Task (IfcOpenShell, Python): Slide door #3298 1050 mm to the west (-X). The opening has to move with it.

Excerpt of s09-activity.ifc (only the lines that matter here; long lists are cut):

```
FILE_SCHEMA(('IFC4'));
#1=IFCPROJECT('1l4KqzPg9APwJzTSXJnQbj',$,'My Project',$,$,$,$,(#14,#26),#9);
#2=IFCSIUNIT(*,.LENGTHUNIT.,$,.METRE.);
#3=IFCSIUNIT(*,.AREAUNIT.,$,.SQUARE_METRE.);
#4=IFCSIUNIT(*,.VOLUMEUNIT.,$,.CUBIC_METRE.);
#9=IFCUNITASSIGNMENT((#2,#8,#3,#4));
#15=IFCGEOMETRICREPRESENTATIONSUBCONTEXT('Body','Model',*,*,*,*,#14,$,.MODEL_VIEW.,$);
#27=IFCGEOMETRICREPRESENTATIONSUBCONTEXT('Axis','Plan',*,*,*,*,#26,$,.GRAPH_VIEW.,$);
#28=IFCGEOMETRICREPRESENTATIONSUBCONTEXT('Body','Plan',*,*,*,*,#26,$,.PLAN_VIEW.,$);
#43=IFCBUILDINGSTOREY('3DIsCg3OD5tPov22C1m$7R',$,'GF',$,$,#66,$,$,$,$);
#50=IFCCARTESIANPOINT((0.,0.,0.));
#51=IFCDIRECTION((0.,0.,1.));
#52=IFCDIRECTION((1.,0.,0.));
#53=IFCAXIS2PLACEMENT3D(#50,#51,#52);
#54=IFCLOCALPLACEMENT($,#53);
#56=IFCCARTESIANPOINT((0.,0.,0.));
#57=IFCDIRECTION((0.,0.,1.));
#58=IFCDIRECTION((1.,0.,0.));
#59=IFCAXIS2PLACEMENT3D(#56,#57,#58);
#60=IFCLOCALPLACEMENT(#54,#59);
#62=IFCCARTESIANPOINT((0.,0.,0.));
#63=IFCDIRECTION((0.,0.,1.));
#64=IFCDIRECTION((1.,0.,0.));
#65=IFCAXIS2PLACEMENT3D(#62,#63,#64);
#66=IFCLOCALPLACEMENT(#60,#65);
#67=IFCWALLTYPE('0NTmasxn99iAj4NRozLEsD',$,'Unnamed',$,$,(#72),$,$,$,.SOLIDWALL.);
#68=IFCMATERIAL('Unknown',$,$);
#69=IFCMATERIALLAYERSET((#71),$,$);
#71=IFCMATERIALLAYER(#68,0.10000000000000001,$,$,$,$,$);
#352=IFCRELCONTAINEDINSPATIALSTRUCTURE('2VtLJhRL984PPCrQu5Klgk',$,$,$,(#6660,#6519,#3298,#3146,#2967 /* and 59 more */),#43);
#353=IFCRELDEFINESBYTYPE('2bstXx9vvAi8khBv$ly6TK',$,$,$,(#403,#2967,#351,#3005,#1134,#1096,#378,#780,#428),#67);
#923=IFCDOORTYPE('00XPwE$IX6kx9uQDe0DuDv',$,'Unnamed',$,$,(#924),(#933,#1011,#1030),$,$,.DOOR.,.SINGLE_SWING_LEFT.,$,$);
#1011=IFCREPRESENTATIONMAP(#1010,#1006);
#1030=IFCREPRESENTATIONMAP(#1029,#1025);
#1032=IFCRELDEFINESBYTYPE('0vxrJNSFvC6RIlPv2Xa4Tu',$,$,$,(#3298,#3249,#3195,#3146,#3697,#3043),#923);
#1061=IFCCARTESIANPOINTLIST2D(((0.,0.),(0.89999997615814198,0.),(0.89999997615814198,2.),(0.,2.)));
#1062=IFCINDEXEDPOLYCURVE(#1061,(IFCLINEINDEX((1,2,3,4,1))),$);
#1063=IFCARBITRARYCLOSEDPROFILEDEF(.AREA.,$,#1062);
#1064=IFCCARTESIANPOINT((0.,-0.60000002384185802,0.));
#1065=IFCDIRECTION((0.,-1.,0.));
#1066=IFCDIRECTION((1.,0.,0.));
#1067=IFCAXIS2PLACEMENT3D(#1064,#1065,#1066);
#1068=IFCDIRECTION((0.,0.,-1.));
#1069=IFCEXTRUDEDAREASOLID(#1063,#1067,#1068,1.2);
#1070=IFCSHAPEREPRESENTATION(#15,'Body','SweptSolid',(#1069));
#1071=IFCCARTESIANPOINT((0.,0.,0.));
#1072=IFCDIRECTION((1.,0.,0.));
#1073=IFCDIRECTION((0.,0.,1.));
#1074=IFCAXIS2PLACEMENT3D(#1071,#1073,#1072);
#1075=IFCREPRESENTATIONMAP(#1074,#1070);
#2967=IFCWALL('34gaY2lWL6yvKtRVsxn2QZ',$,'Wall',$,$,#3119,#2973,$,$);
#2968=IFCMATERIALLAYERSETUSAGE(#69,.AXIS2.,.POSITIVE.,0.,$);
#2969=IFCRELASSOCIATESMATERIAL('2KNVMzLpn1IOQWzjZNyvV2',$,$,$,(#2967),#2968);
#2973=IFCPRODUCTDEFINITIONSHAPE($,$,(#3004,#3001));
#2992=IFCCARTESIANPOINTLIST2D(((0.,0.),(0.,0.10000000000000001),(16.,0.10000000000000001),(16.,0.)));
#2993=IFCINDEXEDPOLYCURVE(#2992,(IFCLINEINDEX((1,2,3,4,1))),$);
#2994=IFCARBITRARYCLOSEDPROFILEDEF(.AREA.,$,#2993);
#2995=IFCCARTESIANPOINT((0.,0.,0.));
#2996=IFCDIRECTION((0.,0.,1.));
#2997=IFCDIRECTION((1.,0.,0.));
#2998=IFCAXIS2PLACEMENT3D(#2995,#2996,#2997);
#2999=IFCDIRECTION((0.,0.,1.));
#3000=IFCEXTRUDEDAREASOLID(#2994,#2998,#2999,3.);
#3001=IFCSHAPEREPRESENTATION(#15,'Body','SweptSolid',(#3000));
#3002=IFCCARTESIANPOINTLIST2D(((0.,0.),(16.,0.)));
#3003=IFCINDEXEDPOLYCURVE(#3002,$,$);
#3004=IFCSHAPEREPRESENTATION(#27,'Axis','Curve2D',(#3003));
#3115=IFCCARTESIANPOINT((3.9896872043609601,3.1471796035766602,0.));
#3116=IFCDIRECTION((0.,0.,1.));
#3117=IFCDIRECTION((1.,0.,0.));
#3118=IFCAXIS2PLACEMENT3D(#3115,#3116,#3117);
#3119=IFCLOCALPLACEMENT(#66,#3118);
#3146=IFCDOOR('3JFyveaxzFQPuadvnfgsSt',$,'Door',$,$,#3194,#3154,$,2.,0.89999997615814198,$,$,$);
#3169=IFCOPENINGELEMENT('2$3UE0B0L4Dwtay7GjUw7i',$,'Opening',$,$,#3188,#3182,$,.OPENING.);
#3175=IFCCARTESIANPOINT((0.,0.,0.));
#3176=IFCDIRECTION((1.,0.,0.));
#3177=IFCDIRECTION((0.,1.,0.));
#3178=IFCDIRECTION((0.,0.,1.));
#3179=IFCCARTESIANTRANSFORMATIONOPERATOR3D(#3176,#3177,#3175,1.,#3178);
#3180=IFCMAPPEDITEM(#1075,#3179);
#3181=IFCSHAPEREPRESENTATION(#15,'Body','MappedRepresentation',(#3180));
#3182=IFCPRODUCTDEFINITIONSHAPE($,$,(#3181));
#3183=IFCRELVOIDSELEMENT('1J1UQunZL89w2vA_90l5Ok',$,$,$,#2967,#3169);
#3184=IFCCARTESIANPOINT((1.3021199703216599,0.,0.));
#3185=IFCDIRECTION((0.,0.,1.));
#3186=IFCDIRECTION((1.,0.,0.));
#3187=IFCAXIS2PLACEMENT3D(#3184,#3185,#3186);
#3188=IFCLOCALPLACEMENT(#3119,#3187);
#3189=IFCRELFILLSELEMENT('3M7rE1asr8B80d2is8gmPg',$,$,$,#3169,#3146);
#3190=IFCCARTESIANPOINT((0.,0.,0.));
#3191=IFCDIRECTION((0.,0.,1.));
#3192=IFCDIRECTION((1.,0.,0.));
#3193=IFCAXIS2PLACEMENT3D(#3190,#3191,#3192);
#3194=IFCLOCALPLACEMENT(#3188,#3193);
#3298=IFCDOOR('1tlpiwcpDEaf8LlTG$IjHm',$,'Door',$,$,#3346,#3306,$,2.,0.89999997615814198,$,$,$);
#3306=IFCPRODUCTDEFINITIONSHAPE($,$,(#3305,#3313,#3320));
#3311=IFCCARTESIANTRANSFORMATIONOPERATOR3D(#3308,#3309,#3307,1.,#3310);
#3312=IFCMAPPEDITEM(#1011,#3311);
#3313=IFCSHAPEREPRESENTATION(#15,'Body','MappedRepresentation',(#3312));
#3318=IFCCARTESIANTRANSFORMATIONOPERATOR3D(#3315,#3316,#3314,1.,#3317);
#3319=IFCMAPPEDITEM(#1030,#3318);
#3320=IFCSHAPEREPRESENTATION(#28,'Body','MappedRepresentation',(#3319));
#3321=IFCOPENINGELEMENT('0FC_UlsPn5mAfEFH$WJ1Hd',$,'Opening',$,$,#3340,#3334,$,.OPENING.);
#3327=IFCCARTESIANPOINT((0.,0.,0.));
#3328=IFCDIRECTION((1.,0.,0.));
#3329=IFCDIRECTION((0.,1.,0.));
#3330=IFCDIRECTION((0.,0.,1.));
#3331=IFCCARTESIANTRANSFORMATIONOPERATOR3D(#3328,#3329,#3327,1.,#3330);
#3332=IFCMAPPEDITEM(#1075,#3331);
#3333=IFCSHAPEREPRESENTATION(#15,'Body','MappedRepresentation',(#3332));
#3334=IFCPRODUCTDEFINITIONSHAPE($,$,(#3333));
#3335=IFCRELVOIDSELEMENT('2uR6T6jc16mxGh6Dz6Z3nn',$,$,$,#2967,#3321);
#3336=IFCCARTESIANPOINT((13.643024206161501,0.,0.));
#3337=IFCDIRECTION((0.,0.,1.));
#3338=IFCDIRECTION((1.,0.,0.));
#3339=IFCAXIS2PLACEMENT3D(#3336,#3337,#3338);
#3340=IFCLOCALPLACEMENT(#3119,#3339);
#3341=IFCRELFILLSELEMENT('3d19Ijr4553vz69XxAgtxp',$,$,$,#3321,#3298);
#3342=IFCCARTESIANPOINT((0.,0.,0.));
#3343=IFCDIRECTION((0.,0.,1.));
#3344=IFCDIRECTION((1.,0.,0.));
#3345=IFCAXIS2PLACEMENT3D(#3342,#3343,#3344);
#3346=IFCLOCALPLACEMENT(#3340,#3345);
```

```python
import ifcopenshell
import ifcopenshell.api.geometry
import ifcopenshell.util.placement

model = ifcopenshell.open("s09-activity.ifc")

door = model.by_guid("1tlpiwcpDEaf8LlTG$IjHm")
opening = door.FillsVoids[0].RelatingOpeningElement
wall = opening.VoidsElements[0].RelatingBuildingElement

wall_matrix = ifcopenshell.util.placement.get_local_placement(wall.ObjectPlacement)
shift = wall_matrix[:3, 0] * -1.05
before = ifcopenshell.util.placement.get_local_placement(door.ObjectPlacement)[:3, 3].copy()

# The door is placed relative to its opening, so it follows when the opening moves.
matrix = ifcopenshell.util.placement.get_local_placement(opening.ObjectPlacement)
matrix[:3, 3] += shift
ifcopenshell.api.geometry.edit_object_placement(
    model, product=opening, matrix=matrix, is_si=False, should_transform_children=True
)

after = ifcopenshell.util.placement.get_local_placement(door.ObjectPlacement)[:3, 3]
print("door moved by", (after - before).round(3) + 0.0)

model.write("s09-activity_v2.ifc")
```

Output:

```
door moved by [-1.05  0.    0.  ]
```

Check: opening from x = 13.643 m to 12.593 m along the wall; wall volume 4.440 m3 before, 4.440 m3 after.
